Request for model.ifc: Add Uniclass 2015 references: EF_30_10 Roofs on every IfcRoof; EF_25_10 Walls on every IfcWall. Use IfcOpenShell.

First a look at what the model holds.

```python
import ifcopenshell

model = ifcopenshell.open("model.ifc")
print(model.schema)
print("classifications:", [c.Name for c in model.by_type("IfcClassification")])
for ifc_class in ("IfcDoor", "IfcRoof", "IfcStair", "IfcWall", "IfcWindow"):
    print(ifc_class, len(model.by_type(ifc_class)))
```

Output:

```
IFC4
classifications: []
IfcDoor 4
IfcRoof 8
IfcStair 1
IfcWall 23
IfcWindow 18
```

```python
import ifcopenshell
import ifcopenshell.api.classification

model = ifcopenshell.open("model.ifc")

system = ifcopenshell.api.classification.add_classification(model, classification="Uniclass 2015")

codes = {
    "IfcRoof": ("EF_30_10", "Roofs"),
    "IfcWall": ("EF_25_10", "Walls"),
}
for ifc_class, (code, name) in codes.items():
    products = model.by_type(ifc_class)
    ifcopenshell.api.classification.add_reference(
        model, products=products, classification=system, identification=code, name=name
    )
    print(code, len(products))

model.write("model_edited.ifc")
```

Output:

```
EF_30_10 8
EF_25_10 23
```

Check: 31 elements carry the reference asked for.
